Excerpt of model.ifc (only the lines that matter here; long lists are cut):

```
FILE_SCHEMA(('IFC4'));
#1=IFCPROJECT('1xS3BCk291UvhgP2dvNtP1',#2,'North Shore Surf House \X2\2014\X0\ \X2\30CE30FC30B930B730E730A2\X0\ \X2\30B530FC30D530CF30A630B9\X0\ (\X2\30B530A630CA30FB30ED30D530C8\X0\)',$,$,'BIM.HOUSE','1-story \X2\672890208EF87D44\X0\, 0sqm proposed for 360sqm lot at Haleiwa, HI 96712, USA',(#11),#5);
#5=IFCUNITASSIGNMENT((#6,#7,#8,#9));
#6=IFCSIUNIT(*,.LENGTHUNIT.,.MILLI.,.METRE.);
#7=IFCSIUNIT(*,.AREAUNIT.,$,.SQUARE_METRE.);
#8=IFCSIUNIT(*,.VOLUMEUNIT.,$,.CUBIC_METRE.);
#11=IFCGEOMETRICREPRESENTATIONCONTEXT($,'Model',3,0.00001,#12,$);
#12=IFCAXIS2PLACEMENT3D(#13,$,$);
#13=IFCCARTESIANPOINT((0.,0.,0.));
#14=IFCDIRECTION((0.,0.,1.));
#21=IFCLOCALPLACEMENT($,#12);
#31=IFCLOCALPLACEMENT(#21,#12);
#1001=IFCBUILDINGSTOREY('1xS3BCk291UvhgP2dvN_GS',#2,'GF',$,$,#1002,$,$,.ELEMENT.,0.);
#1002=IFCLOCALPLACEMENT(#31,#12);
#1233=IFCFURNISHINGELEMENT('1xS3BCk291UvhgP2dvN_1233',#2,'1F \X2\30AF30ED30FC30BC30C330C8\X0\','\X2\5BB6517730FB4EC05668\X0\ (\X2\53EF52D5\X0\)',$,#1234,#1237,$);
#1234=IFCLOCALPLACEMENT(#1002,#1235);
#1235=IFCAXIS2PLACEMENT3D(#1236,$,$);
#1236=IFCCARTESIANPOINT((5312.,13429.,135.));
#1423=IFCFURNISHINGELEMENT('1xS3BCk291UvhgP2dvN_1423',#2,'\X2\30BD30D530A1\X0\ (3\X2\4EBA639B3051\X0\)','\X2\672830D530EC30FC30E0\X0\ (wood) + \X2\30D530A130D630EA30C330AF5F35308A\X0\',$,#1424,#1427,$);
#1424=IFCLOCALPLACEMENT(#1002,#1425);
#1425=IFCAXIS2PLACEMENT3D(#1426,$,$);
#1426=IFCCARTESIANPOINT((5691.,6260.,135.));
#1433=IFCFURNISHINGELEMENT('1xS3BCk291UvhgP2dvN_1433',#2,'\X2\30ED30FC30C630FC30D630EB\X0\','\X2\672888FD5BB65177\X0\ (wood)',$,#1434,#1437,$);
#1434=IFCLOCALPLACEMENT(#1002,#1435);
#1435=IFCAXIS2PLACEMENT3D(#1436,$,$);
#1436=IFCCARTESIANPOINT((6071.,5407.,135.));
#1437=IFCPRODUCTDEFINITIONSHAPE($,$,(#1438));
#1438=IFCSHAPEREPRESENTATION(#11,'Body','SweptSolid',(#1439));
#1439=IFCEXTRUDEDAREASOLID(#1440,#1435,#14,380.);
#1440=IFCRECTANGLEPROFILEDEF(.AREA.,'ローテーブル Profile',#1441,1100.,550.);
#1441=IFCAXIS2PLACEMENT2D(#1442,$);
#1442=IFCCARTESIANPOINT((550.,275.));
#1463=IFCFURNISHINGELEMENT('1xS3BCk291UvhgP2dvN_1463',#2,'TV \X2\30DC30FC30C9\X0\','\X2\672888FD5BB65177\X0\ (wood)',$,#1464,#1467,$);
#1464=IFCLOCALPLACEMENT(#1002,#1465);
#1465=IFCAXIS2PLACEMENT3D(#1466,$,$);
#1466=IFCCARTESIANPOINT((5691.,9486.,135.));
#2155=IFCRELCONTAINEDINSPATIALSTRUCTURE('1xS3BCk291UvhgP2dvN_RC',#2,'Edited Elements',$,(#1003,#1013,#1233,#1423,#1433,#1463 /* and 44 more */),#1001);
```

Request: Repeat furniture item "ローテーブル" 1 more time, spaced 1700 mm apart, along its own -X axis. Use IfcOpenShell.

```python
import ifcopenshell
import ifcopenshell.api.geometry
import ifcopenshell.api.root
import ifcopenshell.util.element
import ifcopenshell.util.placement
import ifcopenshell.util.unit

model = ifcopenshell.open("model.ifc")
unit_scale = ifcopenshell.util.unit.calculate_unit_scale(model)


def reuse_history(source, copy):
    """copy_class also copies each property set's owner history, people and application; keep the originals."""
    for rel in copy.IsDefinedBy:
        if rel.is_a("IfcRelDefinesByProperties") and (history := rel.RelatingPropertyDefinition.OwnerHistory):
            rel.RelatingPropertyDefinition.OwnerHistory = source.OwnerHistory
            ifcopenshell.util.element.remove_deep2(model, history)


source = model.by_guid("1xS3BCk291UvhgP2dvN_1433")
base = ifcopenshell.util.placement.get_local_placement(source.ObjectPlacement)
step = -base[:3, 0] * 1.7 / unit_scale

for i in range(1, 2):
    copy = ifcopenshell.api.root.copy_class(model, product=source)
    copy.Representation = ifcopenshell.util.element.copy_deep(
        model, source.Representation, exclude=["IfcGeometricRepresentationContext", "IfcRepresentationMap"]
    )
    reuse_history(source, copy)
    matrix = base.copy()
    matrix[:3, 3] += i * step
    print("added at", matrix[:3, 3].round(3) + 0.0)
    ifcopenshell.api.geometry.edit_object_placement(model, product=copy, matrix=matrix, is_si=False)

model.write("model_rev.ifc")
```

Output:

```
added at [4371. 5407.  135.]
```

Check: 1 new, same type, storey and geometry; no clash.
